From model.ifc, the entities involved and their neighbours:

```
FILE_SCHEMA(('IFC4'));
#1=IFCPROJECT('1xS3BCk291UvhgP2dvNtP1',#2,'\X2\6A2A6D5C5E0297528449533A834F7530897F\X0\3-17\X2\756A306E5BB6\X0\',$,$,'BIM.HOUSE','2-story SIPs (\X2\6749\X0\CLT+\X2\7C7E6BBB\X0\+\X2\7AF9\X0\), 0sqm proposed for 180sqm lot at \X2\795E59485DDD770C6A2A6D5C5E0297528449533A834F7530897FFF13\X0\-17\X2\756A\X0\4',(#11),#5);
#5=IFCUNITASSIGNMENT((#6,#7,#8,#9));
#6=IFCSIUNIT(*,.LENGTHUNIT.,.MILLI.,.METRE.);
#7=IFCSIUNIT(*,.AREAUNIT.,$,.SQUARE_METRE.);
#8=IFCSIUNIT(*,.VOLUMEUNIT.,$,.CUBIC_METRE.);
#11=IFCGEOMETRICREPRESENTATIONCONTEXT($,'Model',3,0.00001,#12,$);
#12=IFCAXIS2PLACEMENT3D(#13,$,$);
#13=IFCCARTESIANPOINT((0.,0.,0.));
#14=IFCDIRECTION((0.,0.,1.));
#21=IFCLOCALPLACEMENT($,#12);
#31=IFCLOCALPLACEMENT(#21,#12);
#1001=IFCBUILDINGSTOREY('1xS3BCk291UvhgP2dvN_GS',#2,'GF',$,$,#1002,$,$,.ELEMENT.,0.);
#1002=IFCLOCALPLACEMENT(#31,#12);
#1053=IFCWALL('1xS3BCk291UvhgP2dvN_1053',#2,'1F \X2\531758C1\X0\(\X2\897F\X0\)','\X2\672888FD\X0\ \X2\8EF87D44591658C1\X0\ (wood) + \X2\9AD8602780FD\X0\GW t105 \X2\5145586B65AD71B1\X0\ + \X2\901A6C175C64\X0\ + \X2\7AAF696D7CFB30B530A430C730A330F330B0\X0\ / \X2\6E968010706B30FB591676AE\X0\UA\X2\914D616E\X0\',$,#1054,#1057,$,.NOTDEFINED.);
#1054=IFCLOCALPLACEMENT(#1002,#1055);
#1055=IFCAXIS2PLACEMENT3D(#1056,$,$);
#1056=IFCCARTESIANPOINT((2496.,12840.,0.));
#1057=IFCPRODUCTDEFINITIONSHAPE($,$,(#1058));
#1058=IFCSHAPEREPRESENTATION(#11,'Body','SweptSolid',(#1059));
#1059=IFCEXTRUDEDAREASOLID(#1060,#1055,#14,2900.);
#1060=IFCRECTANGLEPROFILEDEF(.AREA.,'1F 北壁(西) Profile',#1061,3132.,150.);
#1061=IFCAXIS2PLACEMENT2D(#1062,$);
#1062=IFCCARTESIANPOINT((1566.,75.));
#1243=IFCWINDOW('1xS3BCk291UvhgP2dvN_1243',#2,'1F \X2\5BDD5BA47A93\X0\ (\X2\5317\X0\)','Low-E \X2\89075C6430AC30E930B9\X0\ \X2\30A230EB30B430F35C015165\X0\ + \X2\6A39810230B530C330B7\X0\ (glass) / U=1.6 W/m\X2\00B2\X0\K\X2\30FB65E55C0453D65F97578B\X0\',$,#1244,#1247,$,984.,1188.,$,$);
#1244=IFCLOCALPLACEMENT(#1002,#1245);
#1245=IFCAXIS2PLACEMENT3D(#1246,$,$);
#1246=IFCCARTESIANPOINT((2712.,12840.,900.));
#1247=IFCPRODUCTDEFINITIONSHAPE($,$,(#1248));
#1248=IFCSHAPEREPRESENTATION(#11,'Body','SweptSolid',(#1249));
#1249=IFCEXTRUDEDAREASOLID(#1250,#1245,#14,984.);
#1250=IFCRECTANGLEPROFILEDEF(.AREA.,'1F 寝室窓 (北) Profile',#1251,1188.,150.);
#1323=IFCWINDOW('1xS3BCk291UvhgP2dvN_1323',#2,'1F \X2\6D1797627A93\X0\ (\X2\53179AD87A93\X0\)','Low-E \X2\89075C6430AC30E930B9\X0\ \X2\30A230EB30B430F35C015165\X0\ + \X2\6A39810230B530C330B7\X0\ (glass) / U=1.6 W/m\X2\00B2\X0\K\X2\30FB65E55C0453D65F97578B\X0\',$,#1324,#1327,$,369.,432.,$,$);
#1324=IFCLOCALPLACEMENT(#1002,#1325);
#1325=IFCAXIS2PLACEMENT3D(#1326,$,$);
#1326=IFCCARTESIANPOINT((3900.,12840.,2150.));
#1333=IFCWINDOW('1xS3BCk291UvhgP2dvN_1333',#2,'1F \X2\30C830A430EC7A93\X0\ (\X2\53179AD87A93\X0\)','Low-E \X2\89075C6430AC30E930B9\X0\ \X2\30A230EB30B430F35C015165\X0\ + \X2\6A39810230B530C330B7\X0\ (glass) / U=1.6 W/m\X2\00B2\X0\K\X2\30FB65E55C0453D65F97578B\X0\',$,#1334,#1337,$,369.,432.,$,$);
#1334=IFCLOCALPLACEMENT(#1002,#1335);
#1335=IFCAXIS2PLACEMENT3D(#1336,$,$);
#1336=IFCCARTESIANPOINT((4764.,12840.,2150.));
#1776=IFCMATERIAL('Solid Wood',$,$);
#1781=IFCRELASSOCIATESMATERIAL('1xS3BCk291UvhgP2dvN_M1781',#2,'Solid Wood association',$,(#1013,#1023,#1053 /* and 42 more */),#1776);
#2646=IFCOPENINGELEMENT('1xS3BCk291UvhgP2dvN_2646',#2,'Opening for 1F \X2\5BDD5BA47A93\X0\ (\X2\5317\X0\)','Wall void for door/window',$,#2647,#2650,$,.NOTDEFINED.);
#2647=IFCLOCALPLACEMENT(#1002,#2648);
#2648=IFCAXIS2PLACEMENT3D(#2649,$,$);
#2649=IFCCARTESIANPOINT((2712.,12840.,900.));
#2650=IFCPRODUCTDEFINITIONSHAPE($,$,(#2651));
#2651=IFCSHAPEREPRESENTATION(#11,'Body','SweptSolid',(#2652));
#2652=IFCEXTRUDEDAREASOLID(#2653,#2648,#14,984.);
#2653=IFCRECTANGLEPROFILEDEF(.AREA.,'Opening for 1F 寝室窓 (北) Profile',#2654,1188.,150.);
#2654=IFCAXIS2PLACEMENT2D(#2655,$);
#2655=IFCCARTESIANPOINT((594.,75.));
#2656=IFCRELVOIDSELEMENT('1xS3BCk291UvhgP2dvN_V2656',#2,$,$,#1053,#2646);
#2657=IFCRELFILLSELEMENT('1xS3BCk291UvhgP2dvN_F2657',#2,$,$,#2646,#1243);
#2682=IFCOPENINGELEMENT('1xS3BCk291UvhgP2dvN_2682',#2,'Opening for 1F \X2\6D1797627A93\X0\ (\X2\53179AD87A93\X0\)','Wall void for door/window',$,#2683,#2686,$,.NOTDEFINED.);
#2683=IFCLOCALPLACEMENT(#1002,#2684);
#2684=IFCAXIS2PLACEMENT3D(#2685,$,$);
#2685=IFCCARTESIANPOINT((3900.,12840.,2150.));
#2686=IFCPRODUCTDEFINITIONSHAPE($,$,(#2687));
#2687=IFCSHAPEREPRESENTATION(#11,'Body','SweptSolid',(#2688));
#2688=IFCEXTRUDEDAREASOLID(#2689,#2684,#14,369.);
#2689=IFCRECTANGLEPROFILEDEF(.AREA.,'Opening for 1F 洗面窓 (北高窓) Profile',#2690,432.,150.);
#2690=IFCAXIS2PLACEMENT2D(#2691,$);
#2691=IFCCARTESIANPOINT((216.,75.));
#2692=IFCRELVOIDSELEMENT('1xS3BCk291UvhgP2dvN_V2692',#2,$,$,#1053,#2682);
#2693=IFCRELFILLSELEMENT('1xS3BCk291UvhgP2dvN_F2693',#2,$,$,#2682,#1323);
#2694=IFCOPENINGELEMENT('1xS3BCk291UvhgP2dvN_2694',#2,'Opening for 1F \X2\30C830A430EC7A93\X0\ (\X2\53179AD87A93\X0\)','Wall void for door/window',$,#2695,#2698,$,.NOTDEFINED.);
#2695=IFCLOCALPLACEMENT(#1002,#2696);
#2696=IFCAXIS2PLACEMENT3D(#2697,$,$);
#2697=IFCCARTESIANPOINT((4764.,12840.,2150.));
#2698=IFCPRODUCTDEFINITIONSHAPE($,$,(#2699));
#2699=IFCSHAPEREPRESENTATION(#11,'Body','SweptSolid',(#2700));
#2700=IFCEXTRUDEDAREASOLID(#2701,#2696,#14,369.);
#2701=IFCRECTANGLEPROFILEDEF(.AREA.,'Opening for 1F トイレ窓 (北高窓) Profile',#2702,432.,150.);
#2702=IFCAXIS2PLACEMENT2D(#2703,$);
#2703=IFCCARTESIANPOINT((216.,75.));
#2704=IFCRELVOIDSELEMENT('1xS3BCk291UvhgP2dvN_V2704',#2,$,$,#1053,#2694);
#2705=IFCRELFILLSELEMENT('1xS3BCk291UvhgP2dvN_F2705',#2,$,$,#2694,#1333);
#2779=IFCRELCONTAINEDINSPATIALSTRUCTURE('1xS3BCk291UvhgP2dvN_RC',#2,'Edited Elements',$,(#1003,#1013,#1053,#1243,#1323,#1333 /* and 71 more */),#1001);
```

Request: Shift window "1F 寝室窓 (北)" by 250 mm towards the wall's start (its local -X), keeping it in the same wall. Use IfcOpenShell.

```python
import ifcopenshell
import ifcopenshell.api.geometry
import ifcopenshell.util.placement
import ifcopenshell.util.unit

model = ifcopenshell.open("model.ifc")
unit_scale = ifcopenshell.util.unit.calculate_unit_scale(model)

window = model.by_guid("1xS3BCk291UvhgP2dvN_1243")
opening = window.FillsVoids[0].RelatingOpeningElement
wall = opening.VoidsElements[0].RelatingBuildingElement

wall_matrix = ifcopenshell.util.placement.get_local_placement(wall.ObjectPlacement)
shift = wall_matrix[:3, 0] * -0.25 / unit_scale
before = ifcopenshell.util.placement.get_local_placement(window.ObjectPlacement)[:3, 3].copy()

# The window is not placed relative to its opening, so move both.
for product in (opening, window):
    matrix = ifcopenshell.util.placement.get_local_placement(product.ObjectPlacement)
    matrix[:3, 3] += shift
    ifcopenshell.api.geometry.edit_object_placement(model, product=product, matrix=matrix, is_si=False)

after = ifcopenshell.util.placement.get_local_placement(window.ObjectPlacement)[:3, 3]
print("window moved by", (after - before).round(3) + 0.0)

model.write("model-out.ifc")
```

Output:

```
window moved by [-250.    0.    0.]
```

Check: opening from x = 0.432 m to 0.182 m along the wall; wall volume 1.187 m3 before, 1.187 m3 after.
